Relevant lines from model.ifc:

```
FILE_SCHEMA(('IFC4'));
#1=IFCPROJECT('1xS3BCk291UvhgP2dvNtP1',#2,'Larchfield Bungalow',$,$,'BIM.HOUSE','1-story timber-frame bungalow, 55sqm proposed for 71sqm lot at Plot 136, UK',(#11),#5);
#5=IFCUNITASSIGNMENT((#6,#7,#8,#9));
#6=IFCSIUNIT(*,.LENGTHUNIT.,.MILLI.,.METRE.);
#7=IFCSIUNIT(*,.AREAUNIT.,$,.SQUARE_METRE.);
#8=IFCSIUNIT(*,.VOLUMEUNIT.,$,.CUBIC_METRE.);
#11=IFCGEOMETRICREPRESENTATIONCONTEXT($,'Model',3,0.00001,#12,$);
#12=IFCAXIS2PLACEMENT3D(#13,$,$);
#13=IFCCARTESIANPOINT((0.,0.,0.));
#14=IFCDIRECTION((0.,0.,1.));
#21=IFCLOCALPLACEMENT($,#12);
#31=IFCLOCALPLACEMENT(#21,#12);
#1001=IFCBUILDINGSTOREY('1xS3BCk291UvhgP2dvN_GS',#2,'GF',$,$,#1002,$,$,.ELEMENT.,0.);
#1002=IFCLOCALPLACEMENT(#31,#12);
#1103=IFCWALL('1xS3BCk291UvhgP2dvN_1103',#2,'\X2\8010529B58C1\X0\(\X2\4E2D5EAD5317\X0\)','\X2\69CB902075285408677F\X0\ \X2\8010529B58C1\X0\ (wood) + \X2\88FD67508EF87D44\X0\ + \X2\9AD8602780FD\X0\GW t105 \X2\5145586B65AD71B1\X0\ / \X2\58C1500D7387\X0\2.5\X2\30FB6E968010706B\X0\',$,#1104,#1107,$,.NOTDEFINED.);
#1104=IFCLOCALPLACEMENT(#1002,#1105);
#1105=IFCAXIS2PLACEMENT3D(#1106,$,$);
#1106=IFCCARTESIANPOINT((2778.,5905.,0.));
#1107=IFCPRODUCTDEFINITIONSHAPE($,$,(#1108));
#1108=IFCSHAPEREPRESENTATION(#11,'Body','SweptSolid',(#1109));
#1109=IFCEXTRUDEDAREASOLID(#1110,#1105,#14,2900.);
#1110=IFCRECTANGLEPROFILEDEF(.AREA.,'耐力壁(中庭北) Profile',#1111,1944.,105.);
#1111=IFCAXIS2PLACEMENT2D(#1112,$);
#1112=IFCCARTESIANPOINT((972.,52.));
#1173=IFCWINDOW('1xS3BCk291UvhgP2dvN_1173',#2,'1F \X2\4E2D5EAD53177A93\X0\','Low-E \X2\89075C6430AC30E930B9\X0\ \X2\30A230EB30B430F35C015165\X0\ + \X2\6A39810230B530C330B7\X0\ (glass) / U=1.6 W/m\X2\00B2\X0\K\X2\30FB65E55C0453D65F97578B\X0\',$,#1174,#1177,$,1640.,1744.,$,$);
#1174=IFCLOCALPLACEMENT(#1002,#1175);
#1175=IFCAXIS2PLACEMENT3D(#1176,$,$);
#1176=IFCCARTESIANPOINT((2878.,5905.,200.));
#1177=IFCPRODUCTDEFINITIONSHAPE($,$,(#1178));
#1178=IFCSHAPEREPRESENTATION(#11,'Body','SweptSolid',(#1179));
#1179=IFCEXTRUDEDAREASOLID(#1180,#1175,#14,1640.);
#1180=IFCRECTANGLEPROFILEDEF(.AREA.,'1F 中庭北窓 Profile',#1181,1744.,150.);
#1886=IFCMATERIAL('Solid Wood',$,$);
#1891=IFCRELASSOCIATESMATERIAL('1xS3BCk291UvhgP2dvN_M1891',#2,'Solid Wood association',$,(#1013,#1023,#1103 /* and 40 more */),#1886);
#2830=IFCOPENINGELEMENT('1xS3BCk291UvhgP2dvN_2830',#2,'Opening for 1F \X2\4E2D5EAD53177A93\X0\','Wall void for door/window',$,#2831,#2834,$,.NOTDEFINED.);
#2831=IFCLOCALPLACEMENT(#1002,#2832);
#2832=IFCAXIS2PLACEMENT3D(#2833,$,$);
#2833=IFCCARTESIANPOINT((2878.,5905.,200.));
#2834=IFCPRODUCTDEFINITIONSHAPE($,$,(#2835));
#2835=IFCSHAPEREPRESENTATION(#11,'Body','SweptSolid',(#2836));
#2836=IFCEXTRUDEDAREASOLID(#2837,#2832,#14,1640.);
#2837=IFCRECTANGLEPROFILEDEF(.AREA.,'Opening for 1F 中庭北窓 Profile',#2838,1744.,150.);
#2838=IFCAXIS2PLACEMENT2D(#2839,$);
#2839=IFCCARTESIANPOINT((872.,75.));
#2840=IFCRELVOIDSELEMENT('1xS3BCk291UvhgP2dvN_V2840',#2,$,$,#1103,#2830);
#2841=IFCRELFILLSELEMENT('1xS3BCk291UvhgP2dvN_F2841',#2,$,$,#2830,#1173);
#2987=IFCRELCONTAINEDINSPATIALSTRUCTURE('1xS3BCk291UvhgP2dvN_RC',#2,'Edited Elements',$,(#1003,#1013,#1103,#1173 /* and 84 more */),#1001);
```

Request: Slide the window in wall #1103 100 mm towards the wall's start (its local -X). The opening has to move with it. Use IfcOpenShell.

```python
import ifcopenshell
import ifcopenshell.api.geometry
import ifcopenshell.util.placement
import ifcopenshell.util.unit

model = ifcopenshell.open("model.ifc")
unit_scale = ifcopenshell.util.unit.calculate_unit_scale(model)

window = model.by_guid("1xS3BCk291UvhgP2dvN_1173")
opening = window.FillsVoids[0].RelatingOpeningElement
wall = opening.VoidsElements[0].RelatingBuildingElement

wall_matrix = ifcopenshell.util.placement.get_local_placement(wall.ObjectPlacement)
shift = wall_matrix[:3, 0] * -0.1 / unit_scale
before = ifcopenshell.util.placement.get_local_placement(window.ObjectPlacement)[:3, 3].copy()

# The window is not placed relative to its opening, so move both.
for product in (opening, window):
    matrix = ifcopenshell.util.placement.get_local_placement(product.ObjectPlacement)
    matrix[:3, 3] += shift
    ifcopenshell.api.geometry.edit_object_placement(model, product=product, matrix=matrix, is_si=False)

after = ifcopenshell.util.placement.get_local_placement(window.ObjectPlacement)[:3, 3]
print("window moved by", (after - before).round(3) + 0.0)

model.write("model_edited.ifc")
```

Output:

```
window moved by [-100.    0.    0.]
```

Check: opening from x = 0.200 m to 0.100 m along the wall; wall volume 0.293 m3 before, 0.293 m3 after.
